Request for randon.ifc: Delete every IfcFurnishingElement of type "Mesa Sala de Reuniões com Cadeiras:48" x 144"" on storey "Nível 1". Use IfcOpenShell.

First a look at what the model holds.

```python
import ifcopenshell
import ifcopenshell.util.element

model = ifcopenshell.open("randon.ifc")
print(model.schema)
storey = next(s for s in model.by_type("IfcBuildingStorey") if s.Name == "Nível 1")
furniture = [e for e in ifcopenshell.util.element.get_decomposition(storey) if e.is_a("IfcFurnishingElement")]
seen = {}
for e in furniture:
    element_type = ifcopenshell.util.element.get_type(e)
    name = element_type.Name if element_type not in (None, e) else None
    seen[name] = seen.get(name, 0) + 1
for name, count in sorted(seen.items(), key=str):
    print(count, "x", name)
```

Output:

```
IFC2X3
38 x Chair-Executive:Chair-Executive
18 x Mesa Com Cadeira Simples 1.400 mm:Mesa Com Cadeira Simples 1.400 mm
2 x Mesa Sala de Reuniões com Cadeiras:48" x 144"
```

```python
import ifcopenshell
import ifcopenshell.api.root
import ifcopenshell.util.element

model = ifcopenshell.open("randon.ifc")

storey = next(s for s in model.by_type("IfcBuildingStorey") if s.Name == "Nível 1")
furniture = [e for e in ifcopenshell.util.element.get_decomposition(storey) if e.is_a("IfcFurnishingElement")]
targets = [e for e in furniture if (t := ifcopenshell.util.element.get_type(e)) not in (None, e) and t.Name == 'Mesa Sala de Reuniões com Cadeiras:48" x 144"']

for e in targets:
    ifcopenshell.api.root.remove_product(model, product=e)
print(len(targets), "removed")

model.write("randon_edited.ifc")
```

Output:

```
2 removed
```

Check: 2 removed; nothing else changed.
